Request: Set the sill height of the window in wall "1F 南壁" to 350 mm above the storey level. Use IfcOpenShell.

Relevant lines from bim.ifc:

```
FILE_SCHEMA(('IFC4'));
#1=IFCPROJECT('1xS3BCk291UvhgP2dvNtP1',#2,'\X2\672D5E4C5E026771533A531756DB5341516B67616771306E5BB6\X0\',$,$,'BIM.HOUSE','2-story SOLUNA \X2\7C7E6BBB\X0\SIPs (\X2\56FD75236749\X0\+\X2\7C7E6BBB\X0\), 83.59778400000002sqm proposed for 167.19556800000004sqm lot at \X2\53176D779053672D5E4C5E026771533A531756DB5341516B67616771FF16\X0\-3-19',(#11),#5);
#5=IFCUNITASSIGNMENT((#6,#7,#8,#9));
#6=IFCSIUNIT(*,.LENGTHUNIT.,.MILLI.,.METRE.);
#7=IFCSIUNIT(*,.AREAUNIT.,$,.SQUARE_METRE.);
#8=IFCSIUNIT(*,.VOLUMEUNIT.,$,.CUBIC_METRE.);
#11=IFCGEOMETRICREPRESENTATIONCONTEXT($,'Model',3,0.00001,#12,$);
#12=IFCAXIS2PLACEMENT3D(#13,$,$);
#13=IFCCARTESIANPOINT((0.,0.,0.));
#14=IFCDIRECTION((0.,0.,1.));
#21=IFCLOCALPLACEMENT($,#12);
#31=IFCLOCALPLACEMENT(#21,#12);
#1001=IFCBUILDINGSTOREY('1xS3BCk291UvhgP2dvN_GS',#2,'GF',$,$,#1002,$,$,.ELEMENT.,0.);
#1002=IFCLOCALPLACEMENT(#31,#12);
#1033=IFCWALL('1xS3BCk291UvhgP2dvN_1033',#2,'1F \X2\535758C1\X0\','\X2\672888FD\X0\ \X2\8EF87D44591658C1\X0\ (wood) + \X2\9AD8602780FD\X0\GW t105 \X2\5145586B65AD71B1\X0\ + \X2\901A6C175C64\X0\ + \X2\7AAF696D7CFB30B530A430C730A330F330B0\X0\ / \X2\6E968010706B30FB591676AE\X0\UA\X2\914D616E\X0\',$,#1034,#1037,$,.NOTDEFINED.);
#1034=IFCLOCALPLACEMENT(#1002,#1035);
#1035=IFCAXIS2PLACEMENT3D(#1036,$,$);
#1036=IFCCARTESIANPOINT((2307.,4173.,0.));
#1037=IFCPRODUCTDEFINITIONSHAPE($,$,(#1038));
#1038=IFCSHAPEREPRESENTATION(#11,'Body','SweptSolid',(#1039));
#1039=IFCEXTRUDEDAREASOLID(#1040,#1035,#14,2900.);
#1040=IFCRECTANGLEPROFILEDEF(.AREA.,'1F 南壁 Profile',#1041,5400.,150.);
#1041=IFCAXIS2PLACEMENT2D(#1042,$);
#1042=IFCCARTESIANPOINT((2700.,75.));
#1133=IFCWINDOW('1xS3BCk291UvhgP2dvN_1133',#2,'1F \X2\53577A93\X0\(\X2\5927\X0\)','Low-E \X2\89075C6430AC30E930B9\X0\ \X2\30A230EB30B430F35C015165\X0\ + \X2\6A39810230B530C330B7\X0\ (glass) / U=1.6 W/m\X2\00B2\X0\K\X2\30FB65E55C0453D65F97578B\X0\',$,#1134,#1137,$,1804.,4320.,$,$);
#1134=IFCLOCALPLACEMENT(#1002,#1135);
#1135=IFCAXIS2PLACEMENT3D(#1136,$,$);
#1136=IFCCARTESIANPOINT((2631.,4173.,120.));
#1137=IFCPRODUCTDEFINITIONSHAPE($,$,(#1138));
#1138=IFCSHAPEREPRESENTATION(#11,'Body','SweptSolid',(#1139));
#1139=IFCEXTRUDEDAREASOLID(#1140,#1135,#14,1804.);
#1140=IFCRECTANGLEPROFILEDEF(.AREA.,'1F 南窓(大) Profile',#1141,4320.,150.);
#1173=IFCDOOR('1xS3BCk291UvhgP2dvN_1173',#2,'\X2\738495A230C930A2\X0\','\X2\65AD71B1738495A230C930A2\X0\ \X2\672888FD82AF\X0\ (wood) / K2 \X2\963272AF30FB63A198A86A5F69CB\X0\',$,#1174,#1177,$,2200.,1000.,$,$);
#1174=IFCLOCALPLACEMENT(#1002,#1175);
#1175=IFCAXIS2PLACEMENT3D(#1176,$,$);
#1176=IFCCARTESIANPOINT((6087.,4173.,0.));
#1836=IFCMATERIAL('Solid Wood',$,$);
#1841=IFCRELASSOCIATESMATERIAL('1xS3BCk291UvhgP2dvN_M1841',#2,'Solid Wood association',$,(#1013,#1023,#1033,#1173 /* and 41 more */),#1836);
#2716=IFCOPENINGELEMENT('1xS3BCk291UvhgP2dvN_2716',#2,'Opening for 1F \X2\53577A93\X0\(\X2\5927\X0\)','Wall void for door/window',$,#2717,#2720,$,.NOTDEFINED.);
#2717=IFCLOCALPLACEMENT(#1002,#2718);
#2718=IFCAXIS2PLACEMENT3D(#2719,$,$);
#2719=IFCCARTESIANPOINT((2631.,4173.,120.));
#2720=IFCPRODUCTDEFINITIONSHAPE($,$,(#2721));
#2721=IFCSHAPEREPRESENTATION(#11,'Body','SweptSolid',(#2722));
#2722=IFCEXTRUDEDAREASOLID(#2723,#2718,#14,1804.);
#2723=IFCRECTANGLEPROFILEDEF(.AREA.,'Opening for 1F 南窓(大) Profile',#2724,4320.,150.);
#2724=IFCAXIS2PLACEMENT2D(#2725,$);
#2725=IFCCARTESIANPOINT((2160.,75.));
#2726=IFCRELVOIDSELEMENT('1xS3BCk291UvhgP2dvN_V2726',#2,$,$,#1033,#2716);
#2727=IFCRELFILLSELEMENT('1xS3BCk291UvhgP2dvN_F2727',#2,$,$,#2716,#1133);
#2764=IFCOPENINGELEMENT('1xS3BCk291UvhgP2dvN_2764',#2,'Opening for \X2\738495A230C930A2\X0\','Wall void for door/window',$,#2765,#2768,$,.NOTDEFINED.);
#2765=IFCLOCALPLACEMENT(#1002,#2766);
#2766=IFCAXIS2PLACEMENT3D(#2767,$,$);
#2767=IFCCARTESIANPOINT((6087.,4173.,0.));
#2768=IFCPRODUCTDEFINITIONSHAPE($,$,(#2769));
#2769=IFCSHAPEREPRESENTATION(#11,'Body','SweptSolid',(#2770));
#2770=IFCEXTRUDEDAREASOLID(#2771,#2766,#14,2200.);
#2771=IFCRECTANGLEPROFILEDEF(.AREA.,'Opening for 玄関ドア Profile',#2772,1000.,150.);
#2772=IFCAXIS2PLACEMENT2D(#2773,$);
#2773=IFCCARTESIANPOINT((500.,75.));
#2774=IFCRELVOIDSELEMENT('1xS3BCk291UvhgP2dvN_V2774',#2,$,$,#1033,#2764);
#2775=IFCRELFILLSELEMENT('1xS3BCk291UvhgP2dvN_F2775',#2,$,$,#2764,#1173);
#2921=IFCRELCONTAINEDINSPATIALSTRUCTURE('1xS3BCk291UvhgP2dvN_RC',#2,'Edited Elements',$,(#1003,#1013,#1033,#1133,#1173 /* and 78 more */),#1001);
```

```python
import numpy as np
import ifcopenshell
import ifcopenshell.api.geometry
import ifcopenshell.geom
import ifcopenshell.util.element
import ifcopenshell.util.placement
import ifcopenshell.util.shape
import ifcopenshell.util.unit

model = ifcopenshell.open("bim.ifc")
unit_scale = ifcopenshell.util.unit.calculate_unit_scale(model)

window = model.by_guid("1xS3BCk291UvhgP2dvN_1133")
opening = window.FillsVoids[0].RelatingOpeningElement
storey = ifcopenshell.util.element.get_container(window, ifc_class="IfcBuildingStorey")
level = ifcopenshell.util.placement.get_local_placement(storey.ObjectPlacement)[2, 3]

# The opening's origin need not be at the sill, so measure its lowest point.
shape = ifcopenshell.geom.create_shape(ifcopenshell.geom.settings(), opening)
bottom = ifcopenshell.util.shape.get_shape_bottom_elevation(shape, shape.geometry) / unit_scale
dz = level + 350.0 - bottom

shift = np.array([0.0, 0.0, dz])
# The window is not placed relative to its opening, so move both.
for product in (opening, window):
    matrix = ifcopenshell.util.placement.get_local_placement(product.ObjectPlacement)
    matrix[:3, 3] += shift
    ifcopenshell.api.geometry.edit_object_placement(model, product=product, matrix=matrix, is_si=False)

print(f"moved by {dz * unit_scale:+.3f} m")

model.write("bim_updated.ifc")
```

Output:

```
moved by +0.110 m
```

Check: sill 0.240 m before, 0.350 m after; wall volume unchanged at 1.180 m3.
